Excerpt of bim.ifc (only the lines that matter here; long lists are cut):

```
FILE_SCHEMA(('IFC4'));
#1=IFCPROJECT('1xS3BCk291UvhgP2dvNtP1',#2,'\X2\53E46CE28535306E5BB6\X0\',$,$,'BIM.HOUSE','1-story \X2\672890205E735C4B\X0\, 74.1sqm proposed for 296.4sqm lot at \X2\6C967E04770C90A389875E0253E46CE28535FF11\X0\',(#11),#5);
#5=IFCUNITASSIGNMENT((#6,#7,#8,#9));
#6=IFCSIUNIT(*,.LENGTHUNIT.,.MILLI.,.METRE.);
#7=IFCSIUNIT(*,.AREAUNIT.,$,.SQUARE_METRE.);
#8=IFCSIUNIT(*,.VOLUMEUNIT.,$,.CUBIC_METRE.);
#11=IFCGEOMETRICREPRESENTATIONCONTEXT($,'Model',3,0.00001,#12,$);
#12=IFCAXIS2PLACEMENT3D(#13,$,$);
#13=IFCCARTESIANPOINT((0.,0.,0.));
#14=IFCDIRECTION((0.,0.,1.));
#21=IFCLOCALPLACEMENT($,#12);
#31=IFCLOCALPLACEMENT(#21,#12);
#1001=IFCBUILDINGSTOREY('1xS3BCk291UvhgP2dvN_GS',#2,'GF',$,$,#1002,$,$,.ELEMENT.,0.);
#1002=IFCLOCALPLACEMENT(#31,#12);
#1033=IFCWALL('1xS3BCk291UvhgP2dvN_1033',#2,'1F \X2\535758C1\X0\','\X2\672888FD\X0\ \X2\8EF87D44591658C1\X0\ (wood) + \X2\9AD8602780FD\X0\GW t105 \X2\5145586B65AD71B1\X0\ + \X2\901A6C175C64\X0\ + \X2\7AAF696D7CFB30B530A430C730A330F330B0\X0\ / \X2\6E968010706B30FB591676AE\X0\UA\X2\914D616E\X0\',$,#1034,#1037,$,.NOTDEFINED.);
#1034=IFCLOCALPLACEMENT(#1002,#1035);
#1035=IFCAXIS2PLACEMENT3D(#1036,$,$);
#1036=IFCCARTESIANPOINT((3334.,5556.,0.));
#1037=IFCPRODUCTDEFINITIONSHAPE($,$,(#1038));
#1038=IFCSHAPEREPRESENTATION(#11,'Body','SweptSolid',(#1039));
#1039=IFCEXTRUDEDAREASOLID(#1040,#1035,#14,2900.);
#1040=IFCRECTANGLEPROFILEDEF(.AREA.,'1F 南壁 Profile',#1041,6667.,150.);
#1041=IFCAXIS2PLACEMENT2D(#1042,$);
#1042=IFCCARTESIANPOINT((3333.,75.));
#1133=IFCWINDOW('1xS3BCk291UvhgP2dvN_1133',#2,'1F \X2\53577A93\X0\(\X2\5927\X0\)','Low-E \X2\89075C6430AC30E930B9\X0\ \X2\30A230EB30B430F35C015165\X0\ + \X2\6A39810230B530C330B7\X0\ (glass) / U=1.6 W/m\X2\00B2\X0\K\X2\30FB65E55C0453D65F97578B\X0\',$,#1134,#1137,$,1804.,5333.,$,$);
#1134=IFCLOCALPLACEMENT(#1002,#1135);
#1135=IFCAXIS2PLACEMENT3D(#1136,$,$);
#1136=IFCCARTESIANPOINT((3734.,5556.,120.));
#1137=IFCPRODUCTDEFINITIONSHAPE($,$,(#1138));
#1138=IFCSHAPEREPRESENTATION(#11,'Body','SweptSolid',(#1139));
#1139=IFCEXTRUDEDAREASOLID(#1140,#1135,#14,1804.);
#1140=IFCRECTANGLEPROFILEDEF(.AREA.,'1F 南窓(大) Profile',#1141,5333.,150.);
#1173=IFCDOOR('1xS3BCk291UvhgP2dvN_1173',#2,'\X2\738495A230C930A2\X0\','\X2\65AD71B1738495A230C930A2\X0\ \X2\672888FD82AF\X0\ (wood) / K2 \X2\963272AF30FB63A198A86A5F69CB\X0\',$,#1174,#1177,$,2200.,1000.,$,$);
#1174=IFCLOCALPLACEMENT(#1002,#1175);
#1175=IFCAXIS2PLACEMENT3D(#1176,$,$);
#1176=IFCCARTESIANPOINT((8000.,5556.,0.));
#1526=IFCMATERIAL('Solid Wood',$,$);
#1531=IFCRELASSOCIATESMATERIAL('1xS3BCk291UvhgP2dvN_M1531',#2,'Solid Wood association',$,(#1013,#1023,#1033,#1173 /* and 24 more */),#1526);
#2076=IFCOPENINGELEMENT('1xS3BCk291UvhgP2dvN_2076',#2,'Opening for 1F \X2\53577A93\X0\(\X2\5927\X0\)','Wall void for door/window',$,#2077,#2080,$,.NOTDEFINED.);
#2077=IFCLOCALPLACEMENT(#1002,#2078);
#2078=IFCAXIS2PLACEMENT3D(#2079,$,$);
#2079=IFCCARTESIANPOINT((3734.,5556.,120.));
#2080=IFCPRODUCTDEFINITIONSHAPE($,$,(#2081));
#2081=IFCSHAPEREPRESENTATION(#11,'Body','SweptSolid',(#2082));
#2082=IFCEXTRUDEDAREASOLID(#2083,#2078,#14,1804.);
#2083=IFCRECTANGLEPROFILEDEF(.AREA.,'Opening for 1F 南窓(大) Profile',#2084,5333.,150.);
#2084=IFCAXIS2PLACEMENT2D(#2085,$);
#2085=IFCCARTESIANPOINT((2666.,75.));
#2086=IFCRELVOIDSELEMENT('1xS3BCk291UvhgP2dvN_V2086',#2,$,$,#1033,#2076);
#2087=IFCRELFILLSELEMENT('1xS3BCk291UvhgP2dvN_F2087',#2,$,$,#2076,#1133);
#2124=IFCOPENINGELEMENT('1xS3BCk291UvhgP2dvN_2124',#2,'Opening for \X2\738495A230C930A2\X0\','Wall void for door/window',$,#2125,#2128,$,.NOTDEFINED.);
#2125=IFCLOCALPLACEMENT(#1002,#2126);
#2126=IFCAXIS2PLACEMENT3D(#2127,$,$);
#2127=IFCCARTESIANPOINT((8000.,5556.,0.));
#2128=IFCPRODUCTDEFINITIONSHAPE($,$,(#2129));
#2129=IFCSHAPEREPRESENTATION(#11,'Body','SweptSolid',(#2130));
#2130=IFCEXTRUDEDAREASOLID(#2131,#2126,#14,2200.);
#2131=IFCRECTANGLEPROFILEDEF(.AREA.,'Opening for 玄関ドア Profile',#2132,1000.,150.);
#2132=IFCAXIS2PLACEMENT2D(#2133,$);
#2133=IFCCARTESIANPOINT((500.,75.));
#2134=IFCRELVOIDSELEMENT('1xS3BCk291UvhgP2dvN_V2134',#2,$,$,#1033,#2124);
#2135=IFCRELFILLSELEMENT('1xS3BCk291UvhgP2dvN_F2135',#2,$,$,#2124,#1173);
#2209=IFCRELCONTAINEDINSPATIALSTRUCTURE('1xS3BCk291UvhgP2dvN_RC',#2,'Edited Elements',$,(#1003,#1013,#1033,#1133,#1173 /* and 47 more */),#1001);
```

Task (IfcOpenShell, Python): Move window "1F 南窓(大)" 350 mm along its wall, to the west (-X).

```python
import ifcopenshell
import ifcopenshell.api.geometry
import ifcopenshell.util.placement
import ifcopenshell.util.unit

model = ifcopenshell.open("bim.ifc")
unit_scale = ifcopenshell.util.unit.calculate_unit_scale(model)

window = model.by_guid("1xS3BCk291UvhgP2dvN_1133")
opening = window.FillsVoids[0].RelatingOpeningElement
wall = opening.VoidsElements[0].RelatingBuildingElement

wall_matrix = ifcopenshell.util.placement.get_local_placement(wall.ObjectPlacement)
shift = wall_matrix[:3, 0] * -0.35 / unit_scale
before = ifcopenshell.util.placement.get_local_placement(window.ObjectPlacement)[:3, 3].copy()

# The window is not placed relative to its opening, so move both.
for product in (opening, window):
    matrix = ifcopenshell.util.placement.get_local_placement(product.ObjectPlacement)
    matrix[:3, 3] += shift
    ifcopenshell.api.geometry.edit_object_placement(model, product=product, matrix=matrix, is_si=False)

after = ifcopenshell.util.placement.get_local_placement(window.ObjectPlacement)[:3, 3]
print("window moved by", (after - before).round(3) + 0.0)

model.write("bim_updated.ifc")
```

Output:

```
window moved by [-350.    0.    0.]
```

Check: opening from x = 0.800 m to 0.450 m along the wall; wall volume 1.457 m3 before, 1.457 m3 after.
